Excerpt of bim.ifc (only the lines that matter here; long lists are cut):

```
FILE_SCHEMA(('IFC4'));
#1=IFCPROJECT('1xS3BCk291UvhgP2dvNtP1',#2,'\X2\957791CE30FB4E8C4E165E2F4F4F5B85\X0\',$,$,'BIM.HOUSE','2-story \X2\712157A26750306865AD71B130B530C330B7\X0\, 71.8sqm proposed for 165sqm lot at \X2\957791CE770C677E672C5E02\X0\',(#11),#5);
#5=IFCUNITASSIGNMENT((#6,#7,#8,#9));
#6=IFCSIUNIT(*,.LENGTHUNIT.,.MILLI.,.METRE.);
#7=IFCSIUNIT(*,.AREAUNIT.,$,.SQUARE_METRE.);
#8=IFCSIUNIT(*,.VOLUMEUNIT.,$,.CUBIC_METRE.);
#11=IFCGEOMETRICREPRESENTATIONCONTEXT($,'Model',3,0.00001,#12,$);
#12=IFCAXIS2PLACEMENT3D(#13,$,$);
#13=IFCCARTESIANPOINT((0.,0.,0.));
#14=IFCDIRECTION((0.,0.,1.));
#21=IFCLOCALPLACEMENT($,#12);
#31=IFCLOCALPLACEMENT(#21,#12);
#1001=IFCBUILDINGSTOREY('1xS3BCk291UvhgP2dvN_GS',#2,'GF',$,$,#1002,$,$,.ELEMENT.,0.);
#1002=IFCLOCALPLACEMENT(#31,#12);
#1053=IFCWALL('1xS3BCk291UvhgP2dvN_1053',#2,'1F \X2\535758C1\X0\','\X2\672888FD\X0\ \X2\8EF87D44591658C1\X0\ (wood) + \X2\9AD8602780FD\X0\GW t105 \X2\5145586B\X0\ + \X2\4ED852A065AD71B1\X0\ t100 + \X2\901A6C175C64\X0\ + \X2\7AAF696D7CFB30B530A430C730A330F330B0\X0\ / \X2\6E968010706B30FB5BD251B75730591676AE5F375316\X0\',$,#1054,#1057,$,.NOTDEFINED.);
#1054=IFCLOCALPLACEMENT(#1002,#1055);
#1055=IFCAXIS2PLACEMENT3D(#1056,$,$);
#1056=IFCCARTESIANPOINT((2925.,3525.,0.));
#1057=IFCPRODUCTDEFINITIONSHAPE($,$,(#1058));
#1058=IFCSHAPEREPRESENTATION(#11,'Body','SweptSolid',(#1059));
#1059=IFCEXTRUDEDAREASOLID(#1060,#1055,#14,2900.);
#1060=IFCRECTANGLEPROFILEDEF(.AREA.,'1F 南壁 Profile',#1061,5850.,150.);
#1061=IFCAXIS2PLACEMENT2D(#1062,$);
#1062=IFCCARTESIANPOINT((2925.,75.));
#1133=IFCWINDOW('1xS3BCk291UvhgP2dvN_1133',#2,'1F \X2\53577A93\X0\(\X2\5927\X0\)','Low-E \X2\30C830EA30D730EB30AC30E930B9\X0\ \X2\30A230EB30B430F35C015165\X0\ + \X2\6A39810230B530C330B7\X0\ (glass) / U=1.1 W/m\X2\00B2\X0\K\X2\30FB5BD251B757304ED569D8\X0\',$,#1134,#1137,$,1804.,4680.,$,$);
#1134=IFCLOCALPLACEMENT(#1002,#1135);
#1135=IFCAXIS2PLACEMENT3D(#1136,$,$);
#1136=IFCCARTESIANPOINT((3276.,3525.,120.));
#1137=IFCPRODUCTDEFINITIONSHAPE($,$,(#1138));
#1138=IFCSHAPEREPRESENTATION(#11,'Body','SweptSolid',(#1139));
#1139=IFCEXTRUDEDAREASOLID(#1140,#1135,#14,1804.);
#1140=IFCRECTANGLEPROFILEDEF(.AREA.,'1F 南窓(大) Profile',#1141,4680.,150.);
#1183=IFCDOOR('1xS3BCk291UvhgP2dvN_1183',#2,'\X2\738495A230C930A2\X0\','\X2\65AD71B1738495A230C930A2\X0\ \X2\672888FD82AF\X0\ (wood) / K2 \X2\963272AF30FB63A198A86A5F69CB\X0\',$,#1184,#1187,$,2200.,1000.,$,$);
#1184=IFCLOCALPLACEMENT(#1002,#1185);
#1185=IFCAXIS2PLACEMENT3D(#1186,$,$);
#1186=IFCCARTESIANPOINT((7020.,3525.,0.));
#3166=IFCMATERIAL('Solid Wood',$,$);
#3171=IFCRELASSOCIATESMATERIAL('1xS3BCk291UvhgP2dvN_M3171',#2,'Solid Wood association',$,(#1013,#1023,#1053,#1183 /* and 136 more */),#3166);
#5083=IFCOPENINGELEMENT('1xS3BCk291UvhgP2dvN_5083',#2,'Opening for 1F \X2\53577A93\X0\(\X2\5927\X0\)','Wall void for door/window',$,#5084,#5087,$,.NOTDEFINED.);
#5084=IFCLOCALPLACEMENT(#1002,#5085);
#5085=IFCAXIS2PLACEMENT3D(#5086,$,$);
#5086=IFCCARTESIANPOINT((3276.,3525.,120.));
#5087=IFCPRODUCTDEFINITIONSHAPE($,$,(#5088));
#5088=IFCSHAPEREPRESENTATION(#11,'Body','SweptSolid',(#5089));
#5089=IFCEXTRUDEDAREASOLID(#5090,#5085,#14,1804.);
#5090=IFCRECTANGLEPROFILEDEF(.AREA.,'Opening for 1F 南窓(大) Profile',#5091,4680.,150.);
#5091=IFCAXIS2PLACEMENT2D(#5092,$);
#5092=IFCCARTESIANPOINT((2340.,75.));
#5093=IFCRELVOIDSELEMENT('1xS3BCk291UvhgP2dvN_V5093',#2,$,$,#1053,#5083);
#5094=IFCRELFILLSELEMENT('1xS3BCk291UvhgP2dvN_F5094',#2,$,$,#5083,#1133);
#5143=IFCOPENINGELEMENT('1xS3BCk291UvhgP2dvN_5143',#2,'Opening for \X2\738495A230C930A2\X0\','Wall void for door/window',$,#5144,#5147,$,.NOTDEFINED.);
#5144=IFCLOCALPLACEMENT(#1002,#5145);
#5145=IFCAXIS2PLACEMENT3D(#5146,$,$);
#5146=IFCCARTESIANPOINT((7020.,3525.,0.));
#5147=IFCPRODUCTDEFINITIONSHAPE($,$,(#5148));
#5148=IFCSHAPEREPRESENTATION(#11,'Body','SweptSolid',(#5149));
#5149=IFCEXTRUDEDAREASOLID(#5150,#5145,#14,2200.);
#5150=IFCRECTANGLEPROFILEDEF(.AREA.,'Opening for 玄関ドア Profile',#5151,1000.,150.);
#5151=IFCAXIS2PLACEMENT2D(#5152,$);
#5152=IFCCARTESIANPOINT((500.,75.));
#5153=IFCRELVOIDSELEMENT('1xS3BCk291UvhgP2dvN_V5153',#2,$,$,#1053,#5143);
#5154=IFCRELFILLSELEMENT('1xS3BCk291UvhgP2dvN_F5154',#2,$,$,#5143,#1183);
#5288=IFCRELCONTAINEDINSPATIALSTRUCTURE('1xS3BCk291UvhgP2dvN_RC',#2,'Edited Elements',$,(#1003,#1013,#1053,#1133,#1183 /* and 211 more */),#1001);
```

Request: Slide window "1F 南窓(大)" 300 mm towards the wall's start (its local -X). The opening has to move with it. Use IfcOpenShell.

```python
import ifcopenshell
import ifcopenshell.api.geometry
import ifcopenshell.util.placement
import ifcopenshell.util.unit

model = ifcopenshell.open("bim.ifc")
unit_scale = ifcopenshell.util.unit.calculate_unit_scale(model)

window = model.by_id(1133)
opening = window.FillsVoids[0].RelatingOpeningElement
wall = opening.VoidsElements[0].RelatingBuildingElement

wall_matrix = ifcopenshell.util.placement.get_local_placement(wall.ObjectPlacement)
shift = wall_matrix[:3, 0] * -0.3 / unit_scale
before = ifcopenshell.util.placement.get_local_placement(window.ObjectPlacement)[:3, 3].copy()

# The window is not placed relative to its opening, so move both.
for product in (opening, window):
    matrix = ifcopenshell.util.placement.get_local_placement(product.ObjectPlacement)
    matrix[:3, 3] += shift
    ifcopenshell.api.geometry.edit_object_placement(model, product=product, matrix=matrix, is_si=False)

after = ifcopenshell.util.placement.get_local_placement(window.ObjectPlacement)[:3, 3]
print("window moved by", (after - before).round(3) + 0.0)

model.write("bim-out.ifc")
```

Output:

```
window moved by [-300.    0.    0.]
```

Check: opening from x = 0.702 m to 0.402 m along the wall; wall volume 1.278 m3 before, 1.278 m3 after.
